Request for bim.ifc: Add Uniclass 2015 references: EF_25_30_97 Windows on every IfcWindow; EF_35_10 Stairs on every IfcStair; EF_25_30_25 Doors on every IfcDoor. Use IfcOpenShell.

First a look at what the model holds.

```python
import ifcopenshell

model = ifcopenshell.open("bim.ifc")
print(model.schema)
print("classifications:", [c.Name for c in model.by_type("IfcClassification")])
for ifc_class in ("IfcDoor", "IfcRoof", "IfcStair", "IfcWall", "IfcWindow"):
    print(ifc_class, len(model.by_type(ifc_class)))
```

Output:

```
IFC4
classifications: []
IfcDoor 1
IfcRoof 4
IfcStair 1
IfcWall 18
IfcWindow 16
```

```python
import ifcopenshell
import ifcopenshell.api.classification

model = ifcopenshell.open("bim.ifc")

system = ifcopenshell.api.classification.add_classification(model, classification="Uniclass 2015")

codes = {
    "IfcWindow": ("EF_25_30_97", "Windows"),
    "IfcStair": ("EF_35_10", "Stairs"),
    "IfcDoor": ("EF_25_30_25", "Doors"),
}
for ifc_class, (code, name) in codes.items():
    products = model.by_type(ifc_class)
    ifcopenshell.api.classification.add_reference(
        model, products=products, classification=system, identification=code, name=name
    )
    print(code, len(products))

model.write("bim-out.ifc")
```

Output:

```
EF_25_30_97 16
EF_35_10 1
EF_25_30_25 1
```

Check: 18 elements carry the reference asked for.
